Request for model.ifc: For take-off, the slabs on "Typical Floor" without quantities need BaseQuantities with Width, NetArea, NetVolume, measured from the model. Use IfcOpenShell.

First a look at what the model holds.

```python
import ifcopenshell
import ifcopenshell.util.element
import ifcopenshell.util.unit

model = ifcopenshell.open("model.ifc")
print(model.schema)
for unit_type in ("LENGTHUNIT", "AREAUNIT", "VOLUMEUNIT"):
    print(unit_type, ifcopenshell.util.unit.calculate_unit_scale(model, unit_type))
storey = next(s for s in model.by_type("IfcBuildingStorey") if s.Name == "Typical Floor")
slabs = [e for e in ifcopenshell.util.element.get_decomposition(storey) if e.is_a("IfcSlab")]
for e in sorted(slabs, key=lambda e: e.id()):
    print(e.id(), e.is_a(), e.Name, list(ifcopenshell.util.element.get_psets(e, qtos_only=True)), sep=" | ")
```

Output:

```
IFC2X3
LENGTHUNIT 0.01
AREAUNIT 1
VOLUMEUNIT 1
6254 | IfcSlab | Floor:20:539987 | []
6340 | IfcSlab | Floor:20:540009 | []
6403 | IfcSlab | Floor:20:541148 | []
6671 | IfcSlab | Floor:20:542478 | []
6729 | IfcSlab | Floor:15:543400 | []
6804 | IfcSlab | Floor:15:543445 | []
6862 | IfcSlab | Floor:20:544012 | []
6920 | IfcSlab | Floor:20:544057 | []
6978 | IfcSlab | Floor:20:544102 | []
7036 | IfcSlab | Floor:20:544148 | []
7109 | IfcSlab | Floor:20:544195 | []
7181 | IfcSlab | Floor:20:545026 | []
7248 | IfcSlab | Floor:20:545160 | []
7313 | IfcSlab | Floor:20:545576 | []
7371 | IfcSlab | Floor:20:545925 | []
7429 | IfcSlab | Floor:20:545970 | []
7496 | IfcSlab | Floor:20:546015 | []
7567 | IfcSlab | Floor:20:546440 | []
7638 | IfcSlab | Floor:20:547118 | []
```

```python
import ifcopenshell
import ifcopenshell.api.pset
import ifcopenshell.geom
import ifcopenshell.util.element
import ifcopenshell.util.shape
import ifcopenshell.util.unit

model = ifcopenshell.open("model.ifc")
unit_scale = ifcopenshell.util.unit.calculate_unit_scale(model)
area_scale = ifcopenshell.util.unit.calculate_unit_scale(model, "AREAUNIT")
volume_scale = ifcopenshell.util.unit.calculate_unit_scale(model, "VOLUMEUNIT")
settings = ifcopenshell.geom.settings()

storey = next(s for s in model.by_type("IfcBuildingStorey") if s.Name == "Typical Floor")
slabs = [e for e in ifcopenshell.util.element.get_decomposition(storey) if e.is_a("IfcSlab")]

for e in sorted(slabs, key=lambda e: e.id()):
    if ifcopenshell.util.element.get_psets(e, qtos_only=True, should_inherit=False):
        continue
    # Geometry comes back in metres, in the element's own axes.
    shape = ifcopenshell.geom.create_shape(settings, e)
    values = {
        "Width": ifcopenshell.util.shape.get_z(shape.geometry) / unit_scale,
        "NetArea": ifcopenshell.util.shape.get_footprint_area(shape.geometry) / area_scale,
        "NetVolume": ifcopenshell.util.shape.get_volume(shape.geometry) / volume_scale,
    }
    qto = ifcopenshell.api.pset.add_qto(model, product=e, name="BaseQuantities")
    ifcopenshell.api.pset.edit_qto(model, qto=qto, properties=values)
    print(e.id(), {k: round(v, 3) for k, v in values.items()})

model.write("model_rev.ifc")
```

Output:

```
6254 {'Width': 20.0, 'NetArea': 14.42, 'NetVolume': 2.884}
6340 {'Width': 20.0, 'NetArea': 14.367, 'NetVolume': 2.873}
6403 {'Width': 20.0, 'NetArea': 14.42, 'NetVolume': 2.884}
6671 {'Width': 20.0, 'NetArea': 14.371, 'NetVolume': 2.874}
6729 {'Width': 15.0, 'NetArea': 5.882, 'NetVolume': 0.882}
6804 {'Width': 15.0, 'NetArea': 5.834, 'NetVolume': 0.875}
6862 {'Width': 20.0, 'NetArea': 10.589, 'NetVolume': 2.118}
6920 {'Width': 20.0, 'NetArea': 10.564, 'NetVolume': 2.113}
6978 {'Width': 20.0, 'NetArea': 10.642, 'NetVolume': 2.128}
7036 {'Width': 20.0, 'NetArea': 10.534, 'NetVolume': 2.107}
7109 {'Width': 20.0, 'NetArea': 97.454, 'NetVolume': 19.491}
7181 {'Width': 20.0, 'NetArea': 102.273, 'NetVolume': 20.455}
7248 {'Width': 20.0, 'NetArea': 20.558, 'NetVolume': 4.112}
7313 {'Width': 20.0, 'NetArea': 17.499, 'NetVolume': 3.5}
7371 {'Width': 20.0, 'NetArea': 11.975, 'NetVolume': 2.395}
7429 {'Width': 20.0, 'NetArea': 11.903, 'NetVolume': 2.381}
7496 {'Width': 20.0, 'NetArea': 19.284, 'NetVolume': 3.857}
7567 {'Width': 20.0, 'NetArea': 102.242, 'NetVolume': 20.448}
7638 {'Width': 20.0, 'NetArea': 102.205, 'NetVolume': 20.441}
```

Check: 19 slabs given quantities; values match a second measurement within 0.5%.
